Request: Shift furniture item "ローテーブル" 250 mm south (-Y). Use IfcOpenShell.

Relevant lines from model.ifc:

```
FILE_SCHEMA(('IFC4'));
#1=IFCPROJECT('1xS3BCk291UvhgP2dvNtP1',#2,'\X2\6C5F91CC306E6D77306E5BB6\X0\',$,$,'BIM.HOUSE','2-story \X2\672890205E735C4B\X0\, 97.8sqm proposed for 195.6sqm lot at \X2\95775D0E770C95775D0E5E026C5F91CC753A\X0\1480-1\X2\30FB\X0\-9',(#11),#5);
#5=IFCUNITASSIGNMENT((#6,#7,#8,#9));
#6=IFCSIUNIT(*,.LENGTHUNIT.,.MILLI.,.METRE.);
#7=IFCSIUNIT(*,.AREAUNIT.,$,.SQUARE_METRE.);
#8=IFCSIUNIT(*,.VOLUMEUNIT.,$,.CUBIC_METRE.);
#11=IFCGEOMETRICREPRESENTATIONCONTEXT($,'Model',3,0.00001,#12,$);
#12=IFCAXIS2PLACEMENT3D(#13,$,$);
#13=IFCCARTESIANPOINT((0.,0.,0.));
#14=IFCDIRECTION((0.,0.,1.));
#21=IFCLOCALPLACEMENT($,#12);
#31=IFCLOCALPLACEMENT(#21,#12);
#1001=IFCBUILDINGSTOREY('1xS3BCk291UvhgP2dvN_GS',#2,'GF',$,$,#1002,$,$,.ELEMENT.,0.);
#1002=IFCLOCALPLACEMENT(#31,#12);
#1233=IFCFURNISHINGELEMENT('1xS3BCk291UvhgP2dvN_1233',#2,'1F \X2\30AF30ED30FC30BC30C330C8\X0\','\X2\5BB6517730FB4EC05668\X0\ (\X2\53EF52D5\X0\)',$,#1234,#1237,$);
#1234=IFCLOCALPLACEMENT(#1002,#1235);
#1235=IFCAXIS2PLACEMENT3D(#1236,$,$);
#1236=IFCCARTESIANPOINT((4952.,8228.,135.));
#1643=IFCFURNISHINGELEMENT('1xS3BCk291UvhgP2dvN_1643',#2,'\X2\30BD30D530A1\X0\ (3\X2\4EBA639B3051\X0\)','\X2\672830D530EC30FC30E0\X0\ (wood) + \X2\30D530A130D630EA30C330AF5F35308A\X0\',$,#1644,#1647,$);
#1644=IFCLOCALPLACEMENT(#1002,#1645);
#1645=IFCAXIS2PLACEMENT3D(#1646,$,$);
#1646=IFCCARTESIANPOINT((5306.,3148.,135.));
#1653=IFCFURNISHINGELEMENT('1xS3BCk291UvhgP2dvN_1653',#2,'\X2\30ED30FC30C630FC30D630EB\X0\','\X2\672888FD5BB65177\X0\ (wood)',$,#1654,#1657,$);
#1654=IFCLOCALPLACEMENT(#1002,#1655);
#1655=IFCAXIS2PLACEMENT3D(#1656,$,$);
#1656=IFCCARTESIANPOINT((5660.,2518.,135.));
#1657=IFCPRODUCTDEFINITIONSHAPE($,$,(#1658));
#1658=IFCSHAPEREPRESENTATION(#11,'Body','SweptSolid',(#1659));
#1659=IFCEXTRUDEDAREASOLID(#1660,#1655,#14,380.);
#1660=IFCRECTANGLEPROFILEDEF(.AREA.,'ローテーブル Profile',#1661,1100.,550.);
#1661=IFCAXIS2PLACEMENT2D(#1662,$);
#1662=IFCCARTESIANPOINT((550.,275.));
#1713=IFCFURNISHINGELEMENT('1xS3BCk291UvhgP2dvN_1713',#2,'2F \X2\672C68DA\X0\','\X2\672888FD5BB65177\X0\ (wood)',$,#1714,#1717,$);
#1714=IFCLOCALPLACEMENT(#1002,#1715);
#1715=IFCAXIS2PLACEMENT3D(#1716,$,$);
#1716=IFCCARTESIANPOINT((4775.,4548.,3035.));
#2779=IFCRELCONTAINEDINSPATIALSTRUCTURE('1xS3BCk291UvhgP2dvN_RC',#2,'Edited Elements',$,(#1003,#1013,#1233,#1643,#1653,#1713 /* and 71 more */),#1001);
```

```python
import ifcopenshell
import ifcopenshell.api.geometry
import ifcopenshell.util.placement
import ifcopenshell.util.unit

model = ifcopenshell.open("model.ifc")
unit_scale = ifcopenshell.util.unit.calculate_unit_scale(model)

item = model.by_id(1653)
matrix = ifcopenshell.util.placement.get_local_placement(item.ObjectPlacement)
matrix[1, 3] -= 0.25 / unit_scale
ifcopenshell.api.geometry.edit_object_placement(model, product=item, matrix=matrix, is_si=False)

print(ifcopenshell.util.placement.get_local_placement(item.ObjectPlacement).round(3) + 0.0)

model.write("model_v2.ifc")
```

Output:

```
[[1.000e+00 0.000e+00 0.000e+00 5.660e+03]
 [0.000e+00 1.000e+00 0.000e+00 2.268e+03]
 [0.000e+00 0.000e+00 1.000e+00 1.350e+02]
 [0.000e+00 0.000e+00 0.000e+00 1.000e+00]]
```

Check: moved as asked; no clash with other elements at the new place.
